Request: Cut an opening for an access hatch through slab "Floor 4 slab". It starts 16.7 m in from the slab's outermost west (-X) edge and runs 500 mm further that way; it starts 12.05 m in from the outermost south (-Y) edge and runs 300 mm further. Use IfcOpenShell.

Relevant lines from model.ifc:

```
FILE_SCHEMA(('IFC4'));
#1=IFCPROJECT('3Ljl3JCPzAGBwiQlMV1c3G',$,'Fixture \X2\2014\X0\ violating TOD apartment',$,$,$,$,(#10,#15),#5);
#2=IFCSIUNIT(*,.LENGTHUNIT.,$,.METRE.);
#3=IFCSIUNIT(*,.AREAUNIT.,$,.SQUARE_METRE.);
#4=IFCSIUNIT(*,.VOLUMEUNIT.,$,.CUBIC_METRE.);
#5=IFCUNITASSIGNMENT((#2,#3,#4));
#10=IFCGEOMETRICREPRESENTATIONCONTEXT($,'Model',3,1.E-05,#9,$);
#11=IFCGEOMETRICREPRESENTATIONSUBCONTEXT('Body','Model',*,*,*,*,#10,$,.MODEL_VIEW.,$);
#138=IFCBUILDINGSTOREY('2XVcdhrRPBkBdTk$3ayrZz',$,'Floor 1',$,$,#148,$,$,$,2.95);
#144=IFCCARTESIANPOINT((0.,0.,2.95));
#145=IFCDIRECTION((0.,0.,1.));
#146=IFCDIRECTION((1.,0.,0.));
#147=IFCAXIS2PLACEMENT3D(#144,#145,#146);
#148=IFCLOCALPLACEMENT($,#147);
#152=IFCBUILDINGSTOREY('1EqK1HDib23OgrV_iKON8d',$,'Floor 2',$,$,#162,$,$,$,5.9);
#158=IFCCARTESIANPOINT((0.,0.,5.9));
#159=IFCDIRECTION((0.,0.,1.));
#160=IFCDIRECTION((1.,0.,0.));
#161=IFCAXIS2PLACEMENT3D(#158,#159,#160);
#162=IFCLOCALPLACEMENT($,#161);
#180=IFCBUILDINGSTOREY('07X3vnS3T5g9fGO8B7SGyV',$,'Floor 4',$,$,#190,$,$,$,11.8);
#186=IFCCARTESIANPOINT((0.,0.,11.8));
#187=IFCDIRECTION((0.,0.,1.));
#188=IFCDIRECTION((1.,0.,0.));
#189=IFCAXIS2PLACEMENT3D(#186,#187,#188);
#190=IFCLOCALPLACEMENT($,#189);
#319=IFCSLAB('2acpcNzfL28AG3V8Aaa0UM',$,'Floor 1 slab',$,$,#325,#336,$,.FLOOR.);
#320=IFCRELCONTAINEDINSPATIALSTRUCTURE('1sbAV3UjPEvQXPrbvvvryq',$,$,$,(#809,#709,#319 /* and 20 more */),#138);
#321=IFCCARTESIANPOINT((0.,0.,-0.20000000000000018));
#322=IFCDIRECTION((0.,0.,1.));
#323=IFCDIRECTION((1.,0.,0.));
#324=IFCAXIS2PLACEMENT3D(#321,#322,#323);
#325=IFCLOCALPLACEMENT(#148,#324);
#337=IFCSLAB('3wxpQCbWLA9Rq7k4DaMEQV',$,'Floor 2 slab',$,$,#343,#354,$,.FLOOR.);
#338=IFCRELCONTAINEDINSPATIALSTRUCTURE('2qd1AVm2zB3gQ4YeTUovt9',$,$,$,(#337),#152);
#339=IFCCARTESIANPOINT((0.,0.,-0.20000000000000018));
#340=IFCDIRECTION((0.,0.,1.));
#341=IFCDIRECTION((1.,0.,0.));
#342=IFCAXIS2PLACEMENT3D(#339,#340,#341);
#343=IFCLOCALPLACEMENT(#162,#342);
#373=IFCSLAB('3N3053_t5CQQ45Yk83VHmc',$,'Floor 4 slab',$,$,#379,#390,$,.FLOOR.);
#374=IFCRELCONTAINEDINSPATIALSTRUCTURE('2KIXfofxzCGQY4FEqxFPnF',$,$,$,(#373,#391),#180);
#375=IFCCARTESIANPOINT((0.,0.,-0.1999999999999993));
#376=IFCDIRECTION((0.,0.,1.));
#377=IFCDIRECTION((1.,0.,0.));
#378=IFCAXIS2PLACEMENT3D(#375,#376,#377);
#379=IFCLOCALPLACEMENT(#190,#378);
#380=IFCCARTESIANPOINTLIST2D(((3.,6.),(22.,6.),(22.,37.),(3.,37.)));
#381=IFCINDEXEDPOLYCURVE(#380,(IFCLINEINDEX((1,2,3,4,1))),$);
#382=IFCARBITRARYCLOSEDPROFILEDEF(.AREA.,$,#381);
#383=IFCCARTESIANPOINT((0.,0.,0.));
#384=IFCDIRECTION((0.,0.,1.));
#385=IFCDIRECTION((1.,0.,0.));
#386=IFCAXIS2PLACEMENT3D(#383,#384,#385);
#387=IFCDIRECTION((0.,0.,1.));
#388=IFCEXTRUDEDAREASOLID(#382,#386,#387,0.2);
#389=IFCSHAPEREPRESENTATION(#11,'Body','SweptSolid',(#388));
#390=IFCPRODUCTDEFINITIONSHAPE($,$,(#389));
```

```python
import numpy as np
import ifcopenshell
import ifcopenshell.api.feature
import ifcopenshell.api.geometry
import ifcopenshell.api.root
import ifcopenshell.geom
import ifcopenshell.util.placement
import ifcopenshell.util.representation
import ifcopenshell.util.shape
import ifcopenshell.util.unit

model = ifcopenshell.open("model.ifc")
unit_scale = ifcopenshell.util.unit.calculate_unit_scale(model)
settings = ifcopenshell.geom.settings()


def volume(element):
    """Net volume in cubic metres, openings subtracted."""
    shape = ifcopenshell.geom.create_shape(settings, element)
    return ifcopenshell.util.shape.get_volume(shape.geometry)


slab = model.by_guid("3N3053_t5CQQ45Yk83VHmc")
before = volume(slab)

# Extent in the slab's own axes, in metres. The edges named are its -X and -Y sides.
slab_shape = ifcopenshell.geom.create_shape(settings, slab)
vertices = ifcopenshell.util.shape.get_vertices(slab_shape.geometry)
x_min, y_min, bottom = vertices.min(axis=0)
top = vertices[:, 2].max()

opening = ifcopenshell.api.root.create_entity(model, ifc_class="IfcOpeningElement", name="Access hatch opening", predefined_type="OPENING")
context = ifcopenshell.util.representation.get_context(model, "Model", "Body", "MODEL_VIEW")
width, depth = 0.5, 0.3
outline = [(0.0, 0.0), (width, 0.0), (width, depth), (0.0, depth), (0.0, 0.0)]
# Overshoot both faces by 50 mm so the cut is clean.
shape = ifcopenshell.api.geometry.add_slab_representation(
    model, context=context, depth=top - bottom + 0.1, polyline=outline
)
ifcopenshell.api.geometry.assign_representation(model, product=opening, representation=shape)

matrix = ifcopenshell.util.placement.get_local_placement(slab.ObjectPlacement)
matrix[:, 3] = matrix @ np.append(np.array([x_min + 16.7, y_min + 12.05, bottom - 0.05]) / unit_scale, 1.0)
ifcopenshell.api.geometry.edit_object_placement(model, product=opening, matrix=matrix, is_si=False)
ifcopenshell.api.feature.add_feature(model, feature=opening, element=slab)

after = volume(slab)

print(f"slab volume {before:.3f} -> {after:.3f} m3")

model.write("model-out.ifc")
```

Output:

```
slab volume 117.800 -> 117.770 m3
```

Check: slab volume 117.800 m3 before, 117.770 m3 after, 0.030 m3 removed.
